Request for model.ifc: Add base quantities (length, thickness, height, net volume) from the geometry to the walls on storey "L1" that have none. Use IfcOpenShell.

First a look at what the model holds.

```python
import ifcopenshell
import ifcopenshell.util.element
import ifcopenshell.util.unit

model = ifcopenshell.open("model.ifc")
print(model.schema)
for unit_type in ("LENGTHUNIT", "AREAUNIT", "VOLUMEUNIT"):
    print(unit_type, ifcopenshell.util.unit.calculate_unit_scale(model, unit_type))
storey = next(s for s in model.by_type("IfcBuildingStorey") if s.Name == "L1")
walls = [e for e in ifcopenshell.util.element.get_decomposition(storey) if e.is_a("IfcWall")]
for e in sorted(walls, key=lambda e: e.id()):
    print(e.id(), e.is_a(), e.Name, list(ifcopenshell.util.element.get_psets(e, qtos_only=True)), sep=" | ")
```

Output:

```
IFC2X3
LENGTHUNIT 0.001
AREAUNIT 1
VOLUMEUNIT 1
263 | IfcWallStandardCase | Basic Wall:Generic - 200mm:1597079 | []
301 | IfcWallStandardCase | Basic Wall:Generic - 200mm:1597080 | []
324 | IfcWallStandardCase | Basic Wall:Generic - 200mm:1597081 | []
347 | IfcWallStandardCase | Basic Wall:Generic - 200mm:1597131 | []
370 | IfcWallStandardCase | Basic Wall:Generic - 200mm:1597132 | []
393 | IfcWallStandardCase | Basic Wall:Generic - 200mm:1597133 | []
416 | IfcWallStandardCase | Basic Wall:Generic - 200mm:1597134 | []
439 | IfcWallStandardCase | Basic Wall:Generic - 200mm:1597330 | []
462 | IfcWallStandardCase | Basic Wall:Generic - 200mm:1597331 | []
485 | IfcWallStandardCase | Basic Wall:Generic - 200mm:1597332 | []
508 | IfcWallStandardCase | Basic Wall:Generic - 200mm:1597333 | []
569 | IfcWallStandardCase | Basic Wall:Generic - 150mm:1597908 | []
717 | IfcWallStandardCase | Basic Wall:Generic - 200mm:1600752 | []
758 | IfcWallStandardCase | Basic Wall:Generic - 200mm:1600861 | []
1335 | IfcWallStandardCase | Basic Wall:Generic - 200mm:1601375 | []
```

```python
import ifcopenshell
import ifcopenshell.api.pset
import ifcopenshell.geom
import ifcopenshell.util.element
import ifcopenshell.util.shape
import ifcopenshell.util.unit

model = ifcopenshell.open("model.ifc")
unit_scale = ifcopenshell.util.unit.calculate_unit_scale(model)
volume_scale = ifcopenshell.util.unit.calculate_unit_scale(model, "VOLUMEUNIT")
settings = ifcopenshell.geom.settings()

storey = next(s for s in model.by_type("IfcBuildingStorey") if s.Name == "L1")
walls = [e for e in ifcopenshell.util.element.get_decomposition(storey) if e.is_a("IfcWall")]

for e in sorted(walls, key=lambda e: e.id()):
    if ifcopenshell.util.element.get_psets(e, qtos_only=True, should_inherit=False):
        continue
    # Geometry comes back in metres, in the element's own axes.
    shape = ifcopenshell.geom.create_shape(settings, e)
    values = {
        "Length": ifcopenshell.util.shape.get_x(shape.geometry) / unit_scale,
        "Width": ifcopenshell.util.shape.get_y(shape.geometry) / unit_scale,
        "Height": ifcopenshell.util.shape.get_z(shape.geometry) / unit_scale,
        "NetVolume": ifcopenshell.util.shape.get_volume(shape.geometry) / volume_scale,
    }
    qto = ifcopenshell.api.pset.add_qto(model, product=e, name="BaseQuantities")
    ifcopenshell.api.pset.edit_qto(model, qto=qto, properties=values)
    print(e.id(), {k: round(v, 3) for k, v in values.items()})

model.write("model_edited.ifc")
```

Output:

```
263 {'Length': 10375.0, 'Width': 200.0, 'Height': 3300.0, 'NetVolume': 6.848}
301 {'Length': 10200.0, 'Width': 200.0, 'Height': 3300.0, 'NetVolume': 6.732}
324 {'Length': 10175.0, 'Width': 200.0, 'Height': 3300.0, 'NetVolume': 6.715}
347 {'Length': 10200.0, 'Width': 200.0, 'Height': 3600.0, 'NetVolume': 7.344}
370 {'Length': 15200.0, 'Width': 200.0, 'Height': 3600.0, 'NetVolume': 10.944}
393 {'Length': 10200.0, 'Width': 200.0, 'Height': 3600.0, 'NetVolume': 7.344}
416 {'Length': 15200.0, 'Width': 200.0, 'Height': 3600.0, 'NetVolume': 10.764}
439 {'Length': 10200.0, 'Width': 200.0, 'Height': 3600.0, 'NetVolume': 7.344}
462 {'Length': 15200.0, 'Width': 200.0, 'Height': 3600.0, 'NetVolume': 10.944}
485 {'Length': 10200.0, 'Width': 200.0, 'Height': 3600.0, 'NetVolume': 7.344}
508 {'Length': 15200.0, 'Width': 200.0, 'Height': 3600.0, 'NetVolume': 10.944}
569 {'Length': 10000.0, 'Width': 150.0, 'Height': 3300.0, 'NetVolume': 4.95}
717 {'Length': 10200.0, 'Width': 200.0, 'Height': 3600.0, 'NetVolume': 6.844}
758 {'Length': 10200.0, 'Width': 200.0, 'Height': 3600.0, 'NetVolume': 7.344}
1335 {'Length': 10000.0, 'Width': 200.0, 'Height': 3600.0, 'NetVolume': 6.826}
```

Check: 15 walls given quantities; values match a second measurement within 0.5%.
